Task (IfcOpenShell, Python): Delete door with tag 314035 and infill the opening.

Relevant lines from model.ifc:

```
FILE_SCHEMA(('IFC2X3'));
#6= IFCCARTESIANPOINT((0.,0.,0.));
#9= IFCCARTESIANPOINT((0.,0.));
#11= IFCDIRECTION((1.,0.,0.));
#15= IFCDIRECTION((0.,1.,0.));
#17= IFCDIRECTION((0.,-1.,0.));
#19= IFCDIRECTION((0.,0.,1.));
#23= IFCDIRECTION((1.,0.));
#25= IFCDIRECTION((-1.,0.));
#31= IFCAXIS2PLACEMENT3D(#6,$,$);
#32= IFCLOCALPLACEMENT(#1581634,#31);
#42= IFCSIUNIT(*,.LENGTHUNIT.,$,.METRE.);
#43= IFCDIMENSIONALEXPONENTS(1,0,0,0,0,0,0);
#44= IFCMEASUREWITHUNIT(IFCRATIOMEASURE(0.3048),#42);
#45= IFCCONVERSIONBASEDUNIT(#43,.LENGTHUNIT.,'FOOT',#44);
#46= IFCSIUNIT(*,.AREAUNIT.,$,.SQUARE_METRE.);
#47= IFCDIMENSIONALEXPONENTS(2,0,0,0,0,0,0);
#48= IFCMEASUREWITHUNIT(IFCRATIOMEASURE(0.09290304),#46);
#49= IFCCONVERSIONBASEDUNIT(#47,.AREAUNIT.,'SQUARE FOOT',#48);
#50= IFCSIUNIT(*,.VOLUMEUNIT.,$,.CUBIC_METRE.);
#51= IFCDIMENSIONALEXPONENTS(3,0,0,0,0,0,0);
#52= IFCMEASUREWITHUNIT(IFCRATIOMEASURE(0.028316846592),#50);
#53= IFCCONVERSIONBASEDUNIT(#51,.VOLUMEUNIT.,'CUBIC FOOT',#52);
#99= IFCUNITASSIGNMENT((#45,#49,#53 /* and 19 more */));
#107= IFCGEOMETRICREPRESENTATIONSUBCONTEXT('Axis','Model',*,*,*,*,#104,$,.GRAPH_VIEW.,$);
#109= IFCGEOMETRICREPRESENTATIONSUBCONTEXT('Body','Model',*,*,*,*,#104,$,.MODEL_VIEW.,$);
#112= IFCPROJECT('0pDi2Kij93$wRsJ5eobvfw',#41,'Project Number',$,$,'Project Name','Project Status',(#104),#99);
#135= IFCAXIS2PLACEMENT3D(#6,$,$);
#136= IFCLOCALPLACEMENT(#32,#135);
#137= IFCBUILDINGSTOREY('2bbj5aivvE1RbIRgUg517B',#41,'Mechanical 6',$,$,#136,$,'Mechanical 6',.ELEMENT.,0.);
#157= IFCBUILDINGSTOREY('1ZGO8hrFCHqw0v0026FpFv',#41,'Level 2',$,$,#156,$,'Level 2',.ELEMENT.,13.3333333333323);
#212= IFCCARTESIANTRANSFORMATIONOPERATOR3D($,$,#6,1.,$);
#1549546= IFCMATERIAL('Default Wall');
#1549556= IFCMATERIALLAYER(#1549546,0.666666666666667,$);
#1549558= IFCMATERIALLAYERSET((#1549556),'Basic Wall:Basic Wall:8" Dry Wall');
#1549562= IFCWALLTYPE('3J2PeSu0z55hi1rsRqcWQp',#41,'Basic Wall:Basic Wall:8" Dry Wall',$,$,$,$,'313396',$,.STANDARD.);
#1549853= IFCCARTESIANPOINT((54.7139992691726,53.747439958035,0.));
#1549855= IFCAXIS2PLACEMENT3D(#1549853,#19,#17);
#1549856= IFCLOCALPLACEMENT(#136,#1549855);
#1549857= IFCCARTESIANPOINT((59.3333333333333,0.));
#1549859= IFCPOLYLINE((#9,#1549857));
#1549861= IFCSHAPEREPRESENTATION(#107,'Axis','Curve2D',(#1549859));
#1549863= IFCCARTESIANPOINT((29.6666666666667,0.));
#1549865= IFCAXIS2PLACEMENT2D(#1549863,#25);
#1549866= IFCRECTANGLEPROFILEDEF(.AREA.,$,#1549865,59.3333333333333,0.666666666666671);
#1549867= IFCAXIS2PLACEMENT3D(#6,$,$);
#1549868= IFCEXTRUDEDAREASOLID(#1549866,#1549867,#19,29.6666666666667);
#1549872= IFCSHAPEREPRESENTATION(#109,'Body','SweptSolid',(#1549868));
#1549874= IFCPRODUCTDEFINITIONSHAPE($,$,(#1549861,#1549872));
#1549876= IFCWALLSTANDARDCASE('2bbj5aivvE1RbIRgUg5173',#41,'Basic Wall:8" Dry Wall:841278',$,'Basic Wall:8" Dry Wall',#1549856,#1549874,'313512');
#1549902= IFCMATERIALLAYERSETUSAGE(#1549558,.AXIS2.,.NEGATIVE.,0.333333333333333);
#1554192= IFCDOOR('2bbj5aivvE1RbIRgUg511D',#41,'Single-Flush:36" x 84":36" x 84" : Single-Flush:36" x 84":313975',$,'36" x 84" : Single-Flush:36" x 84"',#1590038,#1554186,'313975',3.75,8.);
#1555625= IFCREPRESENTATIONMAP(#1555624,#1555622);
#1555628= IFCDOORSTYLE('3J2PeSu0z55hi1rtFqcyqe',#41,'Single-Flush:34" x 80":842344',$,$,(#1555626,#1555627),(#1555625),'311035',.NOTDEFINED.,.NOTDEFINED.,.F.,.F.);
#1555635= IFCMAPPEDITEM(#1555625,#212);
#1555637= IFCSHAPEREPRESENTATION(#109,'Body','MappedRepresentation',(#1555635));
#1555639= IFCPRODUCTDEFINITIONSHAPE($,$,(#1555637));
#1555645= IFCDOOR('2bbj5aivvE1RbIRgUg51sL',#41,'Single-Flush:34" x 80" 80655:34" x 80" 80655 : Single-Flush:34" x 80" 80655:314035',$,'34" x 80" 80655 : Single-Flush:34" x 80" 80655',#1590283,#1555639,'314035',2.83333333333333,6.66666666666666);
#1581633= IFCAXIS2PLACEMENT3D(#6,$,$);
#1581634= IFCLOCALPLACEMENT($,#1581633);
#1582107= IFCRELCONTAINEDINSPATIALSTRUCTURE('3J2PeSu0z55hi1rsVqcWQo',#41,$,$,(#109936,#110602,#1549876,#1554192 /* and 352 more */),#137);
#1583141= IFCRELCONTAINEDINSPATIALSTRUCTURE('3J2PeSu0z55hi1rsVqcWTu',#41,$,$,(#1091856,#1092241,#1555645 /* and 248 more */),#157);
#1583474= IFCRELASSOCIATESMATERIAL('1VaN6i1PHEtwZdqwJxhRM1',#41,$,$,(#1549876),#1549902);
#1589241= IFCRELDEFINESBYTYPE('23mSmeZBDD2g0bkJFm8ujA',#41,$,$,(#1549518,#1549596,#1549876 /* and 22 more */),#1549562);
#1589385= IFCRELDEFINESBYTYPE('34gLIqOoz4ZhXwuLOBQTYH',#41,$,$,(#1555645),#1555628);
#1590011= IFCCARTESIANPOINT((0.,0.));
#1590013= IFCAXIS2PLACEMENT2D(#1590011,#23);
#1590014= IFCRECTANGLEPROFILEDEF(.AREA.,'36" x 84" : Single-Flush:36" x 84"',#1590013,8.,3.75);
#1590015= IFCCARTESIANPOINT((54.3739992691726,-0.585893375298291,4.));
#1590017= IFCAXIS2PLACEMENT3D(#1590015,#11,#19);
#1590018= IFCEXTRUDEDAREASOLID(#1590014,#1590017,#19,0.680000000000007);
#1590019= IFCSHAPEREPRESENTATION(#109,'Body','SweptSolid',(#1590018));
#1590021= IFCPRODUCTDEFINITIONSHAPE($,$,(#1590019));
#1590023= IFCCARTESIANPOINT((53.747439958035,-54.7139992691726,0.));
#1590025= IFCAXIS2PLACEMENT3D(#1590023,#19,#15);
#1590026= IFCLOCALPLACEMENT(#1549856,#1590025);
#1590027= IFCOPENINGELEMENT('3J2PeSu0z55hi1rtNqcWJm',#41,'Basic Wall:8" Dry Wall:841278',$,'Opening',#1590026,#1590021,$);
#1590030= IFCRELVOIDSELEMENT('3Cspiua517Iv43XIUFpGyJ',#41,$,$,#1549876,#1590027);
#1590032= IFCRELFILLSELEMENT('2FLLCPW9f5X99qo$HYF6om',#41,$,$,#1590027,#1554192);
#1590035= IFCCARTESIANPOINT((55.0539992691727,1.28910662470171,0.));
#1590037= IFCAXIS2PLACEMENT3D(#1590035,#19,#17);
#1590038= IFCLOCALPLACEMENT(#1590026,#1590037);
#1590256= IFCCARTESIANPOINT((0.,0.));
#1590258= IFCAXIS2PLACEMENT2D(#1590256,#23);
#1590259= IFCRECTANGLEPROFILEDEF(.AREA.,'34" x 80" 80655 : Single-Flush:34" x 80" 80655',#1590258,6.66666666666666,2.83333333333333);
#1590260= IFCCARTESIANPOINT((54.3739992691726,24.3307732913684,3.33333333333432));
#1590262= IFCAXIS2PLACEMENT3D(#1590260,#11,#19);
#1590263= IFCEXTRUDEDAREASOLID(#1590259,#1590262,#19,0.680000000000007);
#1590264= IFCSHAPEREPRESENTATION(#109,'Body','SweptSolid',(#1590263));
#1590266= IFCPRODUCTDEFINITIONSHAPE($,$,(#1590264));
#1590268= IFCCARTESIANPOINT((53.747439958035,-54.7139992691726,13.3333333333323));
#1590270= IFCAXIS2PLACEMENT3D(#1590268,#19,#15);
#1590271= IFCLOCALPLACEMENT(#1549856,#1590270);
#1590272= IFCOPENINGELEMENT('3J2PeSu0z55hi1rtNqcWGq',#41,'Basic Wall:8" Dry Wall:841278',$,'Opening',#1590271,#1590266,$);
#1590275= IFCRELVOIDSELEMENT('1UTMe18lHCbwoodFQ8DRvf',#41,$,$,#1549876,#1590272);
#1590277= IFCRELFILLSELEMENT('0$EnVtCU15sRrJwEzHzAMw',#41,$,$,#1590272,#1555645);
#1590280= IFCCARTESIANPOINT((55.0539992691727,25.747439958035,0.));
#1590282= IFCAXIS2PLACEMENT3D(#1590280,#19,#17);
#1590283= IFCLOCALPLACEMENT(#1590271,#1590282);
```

```python
import ifcopenshell
import ifcopenshell.api.feature
import ifcopenshell.api.root
import ifcopenshell.geom
import ifcopenshell.util.shape

model = ifcopenshell.open("model.ifc")
settings = ifcopenshell.geom.settings()


def volume(element):
    """Net volume in cubic metres, openings subtracted."""
    shape = ifcopenshell.geom.create_shape(settings, element)
    return ifcopenshell.util.shape.get_volume(shape.geometry)


door = model.by_guid("2bbj5aivvE1RbIRgUg51sL")
opening = door.FillsVoids[0].RelatingOpeningElement
wall = opening.VoidsElements[0].RelatingBuildingElement
before = volume(wall)

ifcopenshell.api.root.remove_product(model, product=door)
ifcopenshell.api.feature.remove_feature(model, feature=opening)

after = volume(wall)

print(f"wall volume {before:.3f} -> {after:.3f} m3")

model.write("model_rev.ifc")
```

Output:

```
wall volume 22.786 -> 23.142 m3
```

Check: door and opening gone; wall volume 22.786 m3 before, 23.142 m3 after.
